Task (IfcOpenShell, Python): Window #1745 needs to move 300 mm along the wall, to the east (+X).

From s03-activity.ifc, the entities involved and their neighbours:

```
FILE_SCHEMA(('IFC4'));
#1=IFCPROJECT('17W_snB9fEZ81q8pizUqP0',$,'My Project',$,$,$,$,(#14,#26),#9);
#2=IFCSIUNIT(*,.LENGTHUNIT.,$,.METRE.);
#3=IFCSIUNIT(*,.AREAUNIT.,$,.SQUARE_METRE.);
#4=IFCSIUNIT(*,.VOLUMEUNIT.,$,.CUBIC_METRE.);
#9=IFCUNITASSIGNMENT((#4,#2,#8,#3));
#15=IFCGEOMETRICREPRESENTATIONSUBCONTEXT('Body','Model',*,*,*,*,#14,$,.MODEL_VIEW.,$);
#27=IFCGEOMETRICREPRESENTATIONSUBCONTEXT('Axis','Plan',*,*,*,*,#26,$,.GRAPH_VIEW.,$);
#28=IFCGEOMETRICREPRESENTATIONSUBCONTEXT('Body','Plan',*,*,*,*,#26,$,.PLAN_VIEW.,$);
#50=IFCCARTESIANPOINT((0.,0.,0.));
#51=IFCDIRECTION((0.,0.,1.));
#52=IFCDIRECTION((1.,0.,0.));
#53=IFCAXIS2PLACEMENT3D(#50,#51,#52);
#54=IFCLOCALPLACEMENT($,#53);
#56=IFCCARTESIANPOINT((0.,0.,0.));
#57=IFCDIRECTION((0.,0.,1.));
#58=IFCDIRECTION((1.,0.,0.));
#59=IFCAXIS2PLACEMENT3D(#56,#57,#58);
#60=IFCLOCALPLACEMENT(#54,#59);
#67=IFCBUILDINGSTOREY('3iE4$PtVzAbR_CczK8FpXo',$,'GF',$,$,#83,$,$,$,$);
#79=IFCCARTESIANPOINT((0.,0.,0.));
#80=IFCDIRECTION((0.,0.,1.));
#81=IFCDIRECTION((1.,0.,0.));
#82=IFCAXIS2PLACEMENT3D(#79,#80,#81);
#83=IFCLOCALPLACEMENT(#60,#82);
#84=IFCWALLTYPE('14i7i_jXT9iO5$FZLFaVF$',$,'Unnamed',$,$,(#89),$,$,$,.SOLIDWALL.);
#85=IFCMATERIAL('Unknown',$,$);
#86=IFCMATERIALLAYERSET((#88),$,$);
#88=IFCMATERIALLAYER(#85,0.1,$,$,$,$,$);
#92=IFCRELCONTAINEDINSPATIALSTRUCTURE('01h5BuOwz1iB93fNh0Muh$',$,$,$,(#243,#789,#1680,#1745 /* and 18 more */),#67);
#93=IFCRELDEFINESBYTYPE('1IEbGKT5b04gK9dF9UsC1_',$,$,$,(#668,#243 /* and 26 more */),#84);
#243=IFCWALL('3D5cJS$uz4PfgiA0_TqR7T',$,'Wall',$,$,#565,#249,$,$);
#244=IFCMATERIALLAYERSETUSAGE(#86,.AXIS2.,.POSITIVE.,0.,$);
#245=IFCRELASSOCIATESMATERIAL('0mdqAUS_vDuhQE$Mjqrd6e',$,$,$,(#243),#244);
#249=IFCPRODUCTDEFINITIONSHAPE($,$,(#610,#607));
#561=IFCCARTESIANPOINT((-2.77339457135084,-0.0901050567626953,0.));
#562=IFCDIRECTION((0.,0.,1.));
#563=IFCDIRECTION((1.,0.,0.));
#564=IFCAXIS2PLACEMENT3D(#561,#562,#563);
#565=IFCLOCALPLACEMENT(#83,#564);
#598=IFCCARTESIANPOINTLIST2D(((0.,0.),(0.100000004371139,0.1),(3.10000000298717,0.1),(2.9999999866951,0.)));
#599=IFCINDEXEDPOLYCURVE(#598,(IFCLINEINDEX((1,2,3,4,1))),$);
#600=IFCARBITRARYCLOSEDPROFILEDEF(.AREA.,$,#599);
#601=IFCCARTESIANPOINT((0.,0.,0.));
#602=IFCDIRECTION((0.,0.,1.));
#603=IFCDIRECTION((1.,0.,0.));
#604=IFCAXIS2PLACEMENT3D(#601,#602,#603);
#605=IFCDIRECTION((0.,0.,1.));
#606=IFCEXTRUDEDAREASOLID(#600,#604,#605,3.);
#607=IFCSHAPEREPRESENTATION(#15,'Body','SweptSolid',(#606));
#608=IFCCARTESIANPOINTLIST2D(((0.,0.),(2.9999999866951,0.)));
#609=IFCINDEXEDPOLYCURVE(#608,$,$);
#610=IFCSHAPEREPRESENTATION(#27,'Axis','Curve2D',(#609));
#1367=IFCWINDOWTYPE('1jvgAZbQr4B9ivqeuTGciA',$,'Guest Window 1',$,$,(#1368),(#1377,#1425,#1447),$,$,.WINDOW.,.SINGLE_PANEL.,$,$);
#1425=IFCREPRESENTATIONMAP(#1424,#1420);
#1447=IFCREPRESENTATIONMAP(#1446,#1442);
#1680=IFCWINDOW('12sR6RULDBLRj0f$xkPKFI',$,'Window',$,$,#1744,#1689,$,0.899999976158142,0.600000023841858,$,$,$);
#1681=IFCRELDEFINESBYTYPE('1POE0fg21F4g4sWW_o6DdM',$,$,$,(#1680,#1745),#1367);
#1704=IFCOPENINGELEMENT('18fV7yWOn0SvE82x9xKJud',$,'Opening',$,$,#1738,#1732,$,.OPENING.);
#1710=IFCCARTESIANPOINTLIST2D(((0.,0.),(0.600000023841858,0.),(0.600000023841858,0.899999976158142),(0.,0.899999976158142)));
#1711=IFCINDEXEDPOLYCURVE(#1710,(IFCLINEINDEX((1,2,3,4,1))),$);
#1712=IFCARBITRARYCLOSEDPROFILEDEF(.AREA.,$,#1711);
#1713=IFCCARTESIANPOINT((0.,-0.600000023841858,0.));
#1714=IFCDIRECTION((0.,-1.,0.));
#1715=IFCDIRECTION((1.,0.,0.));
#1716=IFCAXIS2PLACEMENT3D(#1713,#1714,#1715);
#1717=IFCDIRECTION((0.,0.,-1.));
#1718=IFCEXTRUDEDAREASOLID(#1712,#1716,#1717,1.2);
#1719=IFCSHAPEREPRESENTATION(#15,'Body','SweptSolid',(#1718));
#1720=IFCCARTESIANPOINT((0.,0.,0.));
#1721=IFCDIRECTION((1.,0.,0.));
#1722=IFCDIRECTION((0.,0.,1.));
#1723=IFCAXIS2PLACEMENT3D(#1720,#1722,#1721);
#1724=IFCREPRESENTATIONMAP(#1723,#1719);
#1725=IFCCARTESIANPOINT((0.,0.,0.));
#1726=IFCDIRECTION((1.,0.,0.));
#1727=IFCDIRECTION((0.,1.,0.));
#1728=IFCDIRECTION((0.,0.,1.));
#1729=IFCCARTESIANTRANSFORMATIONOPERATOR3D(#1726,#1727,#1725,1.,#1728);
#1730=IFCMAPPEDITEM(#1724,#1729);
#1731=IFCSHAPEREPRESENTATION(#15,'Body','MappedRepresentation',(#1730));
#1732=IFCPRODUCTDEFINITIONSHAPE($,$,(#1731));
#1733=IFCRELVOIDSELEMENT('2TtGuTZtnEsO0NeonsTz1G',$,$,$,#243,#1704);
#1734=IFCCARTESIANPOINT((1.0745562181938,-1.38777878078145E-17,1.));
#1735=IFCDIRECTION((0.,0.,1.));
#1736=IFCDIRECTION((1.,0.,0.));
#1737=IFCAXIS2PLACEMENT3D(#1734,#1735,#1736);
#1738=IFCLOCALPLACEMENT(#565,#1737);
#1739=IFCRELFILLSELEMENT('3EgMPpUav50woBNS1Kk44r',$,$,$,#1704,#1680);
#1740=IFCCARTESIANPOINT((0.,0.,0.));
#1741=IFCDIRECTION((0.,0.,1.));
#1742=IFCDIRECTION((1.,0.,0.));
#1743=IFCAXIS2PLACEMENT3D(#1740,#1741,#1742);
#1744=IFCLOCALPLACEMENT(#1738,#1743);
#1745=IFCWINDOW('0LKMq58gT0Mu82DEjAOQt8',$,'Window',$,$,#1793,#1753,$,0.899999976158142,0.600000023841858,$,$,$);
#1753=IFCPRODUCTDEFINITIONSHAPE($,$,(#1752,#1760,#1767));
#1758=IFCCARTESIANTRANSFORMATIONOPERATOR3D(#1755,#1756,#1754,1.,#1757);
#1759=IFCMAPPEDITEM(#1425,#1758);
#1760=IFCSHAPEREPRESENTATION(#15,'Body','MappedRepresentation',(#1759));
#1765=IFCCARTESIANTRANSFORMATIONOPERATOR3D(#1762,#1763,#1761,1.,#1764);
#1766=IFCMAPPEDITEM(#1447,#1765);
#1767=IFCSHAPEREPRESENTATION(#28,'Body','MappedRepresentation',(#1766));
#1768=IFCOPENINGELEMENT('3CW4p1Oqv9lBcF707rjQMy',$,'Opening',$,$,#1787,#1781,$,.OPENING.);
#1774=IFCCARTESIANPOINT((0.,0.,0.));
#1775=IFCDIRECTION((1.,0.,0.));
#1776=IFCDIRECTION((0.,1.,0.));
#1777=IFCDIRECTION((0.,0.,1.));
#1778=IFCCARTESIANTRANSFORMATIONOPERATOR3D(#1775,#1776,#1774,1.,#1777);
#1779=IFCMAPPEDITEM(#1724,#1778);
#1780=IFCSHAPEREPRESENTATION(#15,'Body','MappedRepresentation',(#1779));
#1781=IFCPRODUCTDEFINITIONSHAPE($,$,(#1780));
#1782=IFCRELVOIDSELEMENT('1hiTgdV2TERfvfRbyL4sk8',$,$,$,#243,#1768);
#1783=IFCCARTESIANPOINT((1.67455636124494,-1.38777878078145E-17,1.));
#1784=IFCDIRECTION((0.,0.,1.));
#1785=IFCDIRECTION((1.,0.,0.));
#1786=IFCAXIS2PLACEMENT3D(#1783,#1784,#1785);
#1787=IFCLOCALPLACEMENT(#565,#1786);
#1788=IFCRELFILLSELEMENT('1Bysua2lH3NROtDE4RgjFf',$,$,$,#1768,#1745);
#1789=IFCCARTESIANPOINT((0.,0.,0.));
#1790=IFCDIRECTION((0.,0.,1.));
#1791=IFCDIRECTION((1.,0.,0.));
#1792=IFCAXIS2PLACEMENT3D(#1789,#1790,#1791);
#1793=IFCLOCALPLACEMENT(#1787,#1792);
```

```python
import ifcopenshell
import ifcopenshell.api.geometry
import ifcopenshell.util.placement
import ifcopenshell.util.unit

model = ifcopenshell.open("s03-activity.ifc")
unit_scale = ifcopenshell.util.unit.calculate_unit_scale(model)

window = model.by_guid("0LKMq58gT0Mu82DEjAOQt8")
opening = window.FillsVoids[0].RelatingOpeningElement
wall = opening.VoidsElements[0].RelatingBuildingElement

wall_matrix = ifcopenshell.util.placement.get_local_placement(wall.ObjectPlacement)
shift = wall_matrix[:3, 0] * 0.3 / unit_scale
before = ifcopenshell.util.placement.get_local_placement(window.ObjectPlacement)[:3, 3].copy()

# The window is placed relative to its opening, so it follows when the opening moves.
matrix = ifcopenshell.util.placement.get_local_placement(opening.ObjectPlacement)
matrix[:3, 3] += shift
ifcopenshell.api.geometry.edit_object_placement(
    model, product=opening, matrix=matrix, is_si=False, should_transform_children=True
)

after = ifcopenshell.util.placement.get_local_placement(window.ObjectPlacement)[:3, 3]
print("window moved by", (after - before).round(3) + 0.0)

model.write("s03-activity_updated.ifc")
```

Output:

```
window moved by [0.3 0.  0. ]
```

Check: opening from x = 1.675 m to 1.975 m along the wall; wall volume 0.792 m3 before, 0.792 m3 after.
